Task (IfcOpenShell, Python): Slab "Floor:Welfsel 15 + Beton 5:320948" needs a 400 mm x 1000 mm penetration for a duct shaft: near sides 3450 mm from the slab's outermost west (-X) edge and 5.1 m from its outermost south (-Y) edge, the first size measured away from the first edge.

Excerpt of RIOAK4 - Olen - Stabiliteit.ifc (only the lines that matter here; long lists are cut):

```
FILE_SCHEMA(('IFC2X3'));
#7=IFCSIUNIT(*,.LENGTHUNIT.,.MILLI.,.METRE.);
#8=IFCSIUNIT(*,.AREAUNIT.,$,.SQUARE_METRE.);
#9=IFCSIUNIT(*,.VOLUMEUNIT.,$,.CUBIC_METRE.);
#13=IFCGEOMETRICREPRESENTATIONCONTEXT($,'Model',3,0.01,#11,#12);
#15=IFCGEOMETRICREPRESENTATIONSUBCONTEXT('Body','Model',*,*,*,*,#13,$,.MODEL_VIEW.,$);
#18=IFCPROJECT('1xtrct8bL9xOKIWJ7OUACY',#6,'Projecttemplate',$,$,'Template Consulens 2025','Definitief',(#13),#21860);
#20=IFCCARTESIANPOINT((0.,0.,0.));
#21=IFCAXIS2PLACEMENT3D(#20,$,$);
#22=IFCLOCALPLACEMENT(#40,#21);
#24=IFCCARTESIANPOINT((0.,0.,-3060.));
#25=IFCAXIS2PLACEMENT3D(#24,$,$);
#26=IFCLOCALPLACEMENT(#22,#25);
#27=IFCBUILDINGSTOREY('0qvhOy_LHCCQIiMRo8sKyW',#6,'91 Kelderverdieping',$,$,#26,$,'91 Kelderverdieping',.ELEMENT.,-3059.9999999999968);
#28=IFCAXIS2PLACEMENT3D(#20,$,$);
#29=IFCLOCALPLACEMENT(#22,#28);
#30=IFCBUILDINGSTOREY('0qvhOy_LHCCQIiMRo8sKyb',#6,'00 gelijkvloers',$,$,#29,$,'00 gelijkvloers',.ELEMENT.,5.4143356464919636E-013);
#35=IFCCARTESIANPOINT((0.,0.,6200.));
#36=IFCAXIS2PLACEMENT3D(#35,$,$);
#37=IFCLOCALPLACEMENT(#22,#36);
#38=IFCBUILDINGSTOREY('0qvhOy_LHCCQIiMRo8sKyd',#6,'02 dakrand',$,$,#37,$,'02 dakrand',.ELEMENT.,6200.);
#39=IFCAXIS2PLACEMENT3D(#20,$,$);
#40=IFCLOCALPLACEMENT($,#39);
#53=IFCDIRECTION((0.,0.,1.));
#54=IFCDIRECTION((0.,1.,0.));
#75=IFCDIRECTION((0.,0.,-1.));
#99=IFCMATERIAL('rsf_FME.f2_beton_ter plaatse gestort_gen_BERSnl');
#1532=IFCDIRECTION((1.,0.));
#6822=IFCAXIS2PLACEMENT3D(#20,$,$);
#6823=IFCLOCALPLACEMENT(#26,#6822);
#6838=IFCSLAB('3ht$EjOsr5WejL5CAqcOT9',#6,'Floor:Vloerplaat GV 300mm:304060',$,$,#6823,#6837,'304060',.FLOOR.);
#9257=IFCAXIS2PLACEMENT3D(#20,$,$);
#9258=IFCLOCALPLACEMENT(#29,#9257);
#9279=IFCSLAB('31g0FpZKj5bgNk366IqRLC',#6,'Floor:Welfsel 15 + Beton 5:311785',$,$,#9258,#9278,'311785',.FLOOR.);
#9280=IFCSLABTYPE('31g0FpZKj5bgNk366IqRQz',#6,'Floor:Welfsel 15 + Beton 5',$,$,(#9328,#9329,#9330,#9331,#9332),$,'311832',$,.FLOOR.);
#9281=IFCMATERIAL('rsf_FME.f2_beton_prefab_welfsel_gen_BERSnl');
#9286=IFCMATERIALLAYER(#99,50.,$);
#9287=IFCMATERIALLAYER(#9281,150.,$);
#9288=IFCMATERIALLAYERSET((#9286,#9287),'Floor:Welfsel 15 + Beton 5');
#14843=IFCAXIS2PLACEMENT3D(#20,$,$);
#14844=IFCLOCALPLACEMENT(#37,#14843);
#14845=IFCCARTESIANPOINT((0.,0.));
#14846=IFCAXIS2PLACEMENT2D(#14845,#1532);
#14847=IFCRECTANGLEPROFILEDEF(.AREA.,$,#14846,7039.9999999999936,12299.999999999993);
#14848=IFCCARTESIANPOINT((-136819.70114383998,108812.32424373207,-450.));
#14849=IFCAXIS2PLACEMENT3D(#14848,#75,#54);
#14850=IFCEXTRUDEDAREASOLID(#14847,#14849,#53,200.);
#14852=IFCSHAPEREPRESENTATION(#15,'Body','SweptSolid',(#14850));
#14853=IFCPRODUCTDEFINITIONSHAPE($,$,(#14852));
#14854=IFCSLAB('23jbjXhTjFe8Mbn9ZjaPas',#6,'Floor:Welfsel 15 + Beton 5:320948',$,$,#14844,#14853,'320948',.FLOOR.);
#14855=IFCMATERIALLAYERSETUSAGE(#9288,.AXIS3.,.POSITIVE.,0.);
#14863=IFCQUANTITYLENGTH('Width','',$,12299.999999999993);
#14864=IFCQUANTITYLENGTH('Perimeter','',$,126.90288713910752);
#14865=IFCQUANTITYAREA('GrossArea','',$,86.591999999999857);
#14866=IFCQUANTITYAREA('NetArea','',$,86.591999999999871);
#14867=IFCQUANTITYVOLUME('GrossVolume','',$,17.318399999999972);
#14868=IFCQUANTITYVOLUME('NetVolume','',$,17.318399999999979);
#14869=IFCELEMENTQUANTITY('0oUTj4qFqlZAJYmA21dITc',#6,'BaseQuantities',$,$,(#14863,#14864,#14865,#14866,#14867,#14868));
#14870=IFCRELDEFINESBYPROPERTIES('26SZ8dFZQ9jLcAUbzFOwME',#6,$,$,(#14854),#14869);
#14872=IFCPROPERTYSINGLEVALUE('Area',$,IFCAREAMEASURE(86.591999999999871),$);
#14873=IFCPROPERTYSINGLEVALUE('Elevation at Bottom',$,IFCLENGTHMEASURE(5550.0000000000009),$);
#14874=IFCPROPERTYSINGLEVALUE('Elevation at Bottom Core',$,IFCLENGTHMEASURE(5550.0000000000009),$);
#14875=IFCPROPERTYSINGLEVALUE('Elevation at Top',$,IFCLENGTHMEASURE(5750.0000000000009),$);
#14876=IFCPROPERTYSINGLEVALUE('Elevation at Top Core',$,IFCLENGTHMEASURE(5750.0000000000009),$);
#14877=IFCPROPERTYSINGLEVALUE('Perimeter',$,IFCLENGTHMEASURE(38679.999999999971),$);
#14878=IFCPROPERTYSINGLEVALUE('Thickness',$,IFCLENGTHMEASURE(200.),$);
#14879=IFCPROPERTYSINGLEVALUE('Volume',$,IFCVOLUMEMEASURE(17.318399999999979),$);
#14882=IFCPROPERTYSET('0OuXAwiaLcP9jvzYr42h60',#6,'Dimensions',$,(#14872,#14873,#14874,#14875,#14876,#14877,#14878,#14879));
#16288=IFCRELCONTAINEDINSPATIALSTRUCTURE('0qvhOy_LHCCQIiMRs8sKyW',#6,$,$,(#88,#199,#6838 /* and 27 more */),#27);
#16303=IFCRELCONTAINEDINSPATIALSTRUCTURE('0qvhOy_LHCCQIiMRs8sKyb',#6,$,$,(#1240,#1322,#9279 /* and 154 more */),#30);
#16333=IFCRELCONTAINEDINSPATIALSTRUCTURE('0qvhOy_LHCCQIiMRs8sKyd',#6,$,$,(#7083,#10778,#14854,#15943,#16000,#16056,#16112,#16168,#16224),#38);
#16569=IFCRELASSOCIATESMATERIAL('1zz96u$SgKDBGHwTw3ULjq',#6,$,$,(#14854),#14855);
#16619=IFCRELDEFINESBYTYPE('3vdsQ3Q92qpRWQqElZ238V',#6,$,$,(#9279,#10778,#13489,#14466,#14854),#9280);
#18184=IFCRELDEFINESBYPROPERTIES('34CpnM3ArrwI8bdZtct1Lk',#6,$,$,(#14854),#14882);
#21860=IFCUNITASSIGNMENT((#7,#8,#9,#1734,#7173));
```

```python
import numpy as np
import ifcopenshell
import ifcopenshell.api.feature
import ifcopenshell.api.geometry
import ifcopenshell.api.pset
import ifcopenshell.api.root
import ifcopenshell.geom
import ifcopenshell.util.element
import ifcopenshell.util.placement
import ifcopenshell.util.representation
import ifcopenshell.util.shape
import ifcopenshell.util.unit

model = ifcopenshell.open("RIOAK4 - Olen - Stabiliteit.ifc")
unit_scale = ifcopenshell.util.unit.calculate_unit_scale(model)
area_scale = ifcopenshell.util.unit.calculate_unit_scale(model, "AREAUNIT")
volume_scale = ifcopenshell.util.unit.calculate_unit_scale(model, "VOLUMEUNIT")
settings = ifcopenshell.geom.settings()


def volume(element):
    """Net volume in cubic metres, openings subtracted."""
    shape = ifcopenshell.geom.create_shape(settings, element)
    return ifcopenshell.util.shape.get_volume(shape.geometry)


slab = model.by_id(14854)
before = volume(slab)

# Extent in the slab's own axes, in metres. The edges named are its -X and -Y sides.
slab_shape = ifcopenshell.geom.create_shape(settings, slab)
vertices = ifcopenshell.util.shape.get_vertices(slab_shape.geometry)
x_min, y_min, bottom = vertices.min(axis=0)
top = vertices[:, 2].max()

opening = ifcopenshell.api.root.create_entity(model, ifc_class="IfcOpeningElement", name="Duct shaft opening")
context = ifcopenshell.util.representation.get_context(model, "Model", "Body", "MODEL_VIEW")
width, depth = 0.4, 1
outline = [(0.0, 0.0), (width, 0.0), (width, depth), (0.0, depth), (0.0, 0.0)]
# Overshoot both faces by 50 mm so the cut is clean.
shape = ifcopenshell.api.geometry.add_slab_representation(
    model, context=context, depth=top - bottom + 0.1, polyline=outline
)
ifcopenshell.api.geometry.assign_representation(model, product=opening, representation=shape)

matrix = ifcopenshell.util.placement.get_local_placement(slab.ObjectPlacement)
matrix[:, 3] = matrix @ np.append(np.array([x_min + 3.45, y_min + 5.1, bottom - 0.05]) / unit_scale, 1.0)
ifcopenshell.api.geometry.edit_object_placement(model, product=opening, matrix=matrix, is_si=False)
ifcopenshell.api.feature.add_feature(model, feature=opening, element=slab)

after = volume(slab)

# Update the slab's stored quantities.
qto = model.by_id(ifcopenshell.util.element.get_pset(slab, "BaseQuantities", should_inherit=False)["id"])
ifcopenshell.api.pset.edit_qto(model, qto=qto, properties={
    "NetArea": after / (top - bottom) / area_scale,
    "NetVolume": after / volume_scale,
})
pset = model.by_id(ifcopenshell.util.element.get_pset(slab, "Dimensions", should_inherit=False)["id"])
ifcopenshell.api.pset.edit_pset(model, pset=pset, properties={
    "Area": model.create_entity("IfcAreaMeasure", after / (top - bottom) / area_scale),
    "Volume": model.create_entity("IfcVolumeMeasure", after / volume_scale),
})

print(f"slab volume {before:.3f} -> {after:.3f} m3")

model.write("RIOAK4 - Olen - Stabiliteit-out.ifc")
```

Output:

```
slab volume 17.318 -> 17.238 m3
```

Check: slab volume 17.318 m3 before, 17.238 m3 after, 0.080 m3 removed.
